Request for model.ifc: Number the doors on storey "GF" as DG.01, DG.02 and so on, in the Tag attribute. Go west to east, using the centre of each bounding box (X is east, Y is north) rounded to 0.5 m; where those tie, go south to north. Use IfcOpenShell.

First a look at what the model holds.

```python
import ifcopenshell
import ifcopenshell.util.element
import ifcopenshell.util.placement

model = ifcopenshell.open("model.ifc")
print(model.schema)
storey = next(s for s in model.by_type("IfcBuildingStorey") if s.Name == "GF")
doors = [e for e in ifcopenshell.util.element.get_decomposition(storey) if e.is_a("IfcDoor")]
for e in sorted(doors, key=lambda e: e.id()):
    origin = ifcopenshell.util.placement.get_local_placement(e.ObjectPlacement)[:3, 3]
    print(e.id(), e.Tag, e.Name, origin.round(2) + 0.0, sep=" | ")
```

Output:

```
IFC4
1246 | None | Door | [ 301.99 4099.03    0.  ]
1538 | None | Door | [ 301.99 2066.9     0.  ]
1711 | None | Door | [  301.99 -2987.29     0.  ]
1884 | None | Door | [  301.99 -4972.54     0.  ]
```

```python
import ifcopenshell
import ifcopenshell.geom
import ifcopenshell.util.element
import ifcopenshell.util.shape

model = ifcopenshell.open("model.ifc")
settings = ifcopenshell.geom.settings()
settings.set("use-world-coords", True)


def centre(element):
    shape = ifcopenshell.geom.create_shape(settings, element)
    return ifcopenshell.util.shape.get_bbox_centroid(shape.geometry)


storey = next(s for s in model.by_type("IfcBuildingStorey") if s.Name == "GF")
doors = [e for e in ifcopenshell.util.element.get_decomposition(storey) if e.is_a("IfcDoor")]

# Insertion points can sit at a corner or the storey origin, so sort by the geometry (in metres).
centres = {e: centre(e) for e in doors}
doors.sort(key=lambda e: (round(centres[e][0] / 0.5), centres[e][1]))

for i, e in enumerate(doors, start=1):
    number = f"DG.{i:02d}"
    e.Tag = number
    print(e.id(), number)

model.write("model_rev.ifc")
```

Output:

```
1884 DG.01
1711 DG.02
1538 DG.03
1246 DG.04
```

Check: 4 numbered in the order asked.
